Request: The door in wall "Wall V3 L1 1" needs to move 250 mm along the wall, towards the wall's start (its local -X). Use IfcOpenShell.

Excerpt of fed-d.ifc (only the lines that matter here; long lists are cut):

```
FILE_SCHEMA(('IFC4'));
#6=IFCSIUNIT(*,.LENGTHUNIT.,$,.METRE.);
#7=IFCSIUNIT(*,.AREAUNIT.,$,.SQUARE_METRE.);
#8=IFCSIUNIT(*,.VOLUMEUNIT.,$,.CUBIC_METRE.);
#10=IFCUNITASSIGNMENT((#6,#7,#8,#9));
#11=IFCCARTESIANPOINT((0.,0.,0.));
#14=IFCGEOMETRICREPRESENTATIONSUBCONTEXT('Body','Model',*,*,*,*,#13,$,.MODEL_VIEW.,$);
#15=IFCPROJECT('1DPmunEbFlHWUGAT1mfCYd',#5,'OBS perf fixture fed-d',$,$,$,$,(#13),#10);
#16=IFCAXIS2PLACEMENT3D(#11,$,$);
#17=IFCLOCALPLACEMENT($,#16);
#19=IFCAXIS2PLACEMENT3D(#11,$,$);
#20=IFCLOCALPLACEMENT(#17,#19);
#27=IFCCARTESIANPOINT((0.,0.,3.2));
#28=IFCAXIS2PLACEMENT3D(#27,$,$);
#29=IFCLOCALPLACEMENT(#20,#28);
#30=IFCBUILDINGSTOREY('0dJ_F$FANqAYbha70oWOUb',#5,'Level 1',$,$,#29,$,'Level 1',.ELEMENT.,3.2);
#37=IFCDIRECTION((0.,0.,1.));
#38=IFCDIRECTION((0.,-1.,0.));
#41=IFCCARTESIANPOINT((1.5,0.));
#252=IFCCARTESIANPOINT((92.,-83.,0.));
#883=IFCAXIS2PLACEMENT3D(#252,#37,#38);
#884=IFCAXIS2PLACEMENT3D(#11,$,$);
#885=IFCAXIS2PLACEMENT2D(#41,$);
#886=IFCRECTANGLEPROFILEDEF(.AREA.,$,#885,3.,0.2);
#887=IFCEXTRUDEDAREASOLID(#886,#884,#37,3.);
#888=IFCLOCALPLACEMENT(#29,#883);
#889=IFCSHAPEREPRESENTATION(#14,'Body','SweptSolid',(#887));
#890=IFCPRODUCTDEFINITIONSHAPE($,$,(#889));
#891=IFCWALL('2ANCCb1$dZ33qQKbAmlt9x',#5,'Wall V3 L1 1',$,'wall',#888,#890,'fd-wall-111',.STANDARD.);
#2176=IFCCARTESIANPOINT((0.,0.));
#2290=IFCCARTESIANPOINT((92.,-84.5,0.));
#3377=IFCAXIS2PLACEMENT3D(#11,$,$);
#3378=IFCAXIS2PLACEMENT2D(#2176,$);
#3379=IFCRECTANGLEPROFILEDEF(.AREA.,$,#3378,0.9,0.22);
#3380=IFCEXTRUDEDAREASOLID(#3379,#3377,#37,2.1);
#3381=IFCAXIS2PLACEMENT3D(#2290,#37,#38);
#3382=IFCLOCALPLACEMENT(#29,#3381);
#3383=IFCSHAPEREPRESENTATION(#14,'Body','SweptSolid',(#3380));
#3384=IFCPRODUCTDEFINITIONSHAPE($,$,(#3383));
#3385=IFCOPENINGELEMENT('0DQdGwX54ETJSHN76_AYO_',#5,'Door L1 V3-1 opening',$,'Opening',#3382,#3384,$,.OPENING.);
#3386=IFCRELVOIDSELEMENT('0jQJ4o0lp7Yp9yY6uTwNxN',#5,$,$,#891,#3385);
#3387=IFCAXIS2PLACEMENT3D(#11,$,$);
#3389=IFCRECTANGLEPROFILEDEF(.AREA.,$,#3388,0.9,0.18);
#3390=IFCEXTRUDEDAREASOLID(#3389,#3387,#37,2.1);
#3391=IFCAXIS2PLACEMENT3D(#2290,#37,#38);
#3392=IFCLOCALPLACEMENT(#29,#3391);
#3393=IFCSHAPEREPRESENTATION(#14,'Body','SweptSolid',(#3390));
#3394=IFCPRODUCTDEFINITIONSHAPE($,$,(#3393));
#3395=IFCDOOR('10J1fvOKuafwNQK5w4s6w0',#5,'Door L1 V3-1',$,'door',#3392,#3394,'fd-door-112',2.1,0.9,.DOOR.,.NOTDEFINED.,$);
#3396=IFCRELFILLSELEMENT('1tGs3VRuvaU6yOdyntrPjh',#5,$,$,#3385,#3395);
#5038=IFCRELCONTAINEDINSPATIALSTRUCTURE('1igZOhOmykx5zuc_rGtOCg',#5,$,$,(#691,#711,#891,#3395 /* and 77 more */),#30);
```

```python
import ifcopenshell
import ifcopenshell.api.geometry
import ifcopenshell.util.placement
import ifcopenshell.util.unit

model = ifcopenshell.open("fed-d.ifc")
unit_scale = ifcopenshell.util.unit.calculate_unit_scale(model)

door = model.by_guid("10J1fvOKuafwNQK5w4s6w0")
opening = door.FillsVoids[0].RelatingOpeningElement
wall = opening.VoidsElements[0].RelatingBuildingElement

wall_matrix = ifcopenshell.util.placement.get_local_placement(wall.ObjectPlacement)
shift = wall_matrix[:3, 0] * -0.25 / unit_scale
before = ifcopenshell.util.placement.get_local_placement(door.ObjectPlacement)[:3, 3].copy()

# The door is not placed relative to its opening, so move both.
for product in (opening, door):
    matrix = ifcopenshell.util.placement.get_local_placement(product.ObjectPlacement)
    matrix[:3, 3] += shift
    ifcopenshell.api.geometry.edit_object_placement(model, product=product, matrix=matrix, is_si=False)

after = ifcopenshell.util.placement.get_local_placement(door.ObjectPlacement)[:3, 3]
print("door moved by", (after - before).round(3) + 0.0)

model.write("fed-d_updated.ifc")
```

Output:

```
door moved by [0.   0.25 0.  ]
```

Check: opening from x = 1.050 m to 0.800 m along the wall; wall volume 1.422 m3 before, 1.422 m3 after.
